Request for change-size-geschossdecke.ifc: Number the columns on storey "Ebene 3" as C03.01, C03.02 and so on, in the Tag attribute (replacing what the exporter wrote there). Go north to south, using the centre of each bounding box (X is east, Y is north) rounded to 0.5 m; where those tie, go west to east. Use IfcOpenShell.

First a look at what the model holds.

```python
import ifcopenshell
import ifcopenshell.util.element
import ifcopenshell.util.placement

model = ifcopenshell.open("change-size-geschossdecke.ifc")
print(model.schema)
storey = next(s for s in model.by_type("IfcBuildingStorey") if s.Name == "Ebene 3")
columns = [e for e in ifcopenshell.util.element.get_decomposition(storey) if e.is_a("IfcColumn")]
for e in sorted(columns, key=lambda e: e.id()):
    origin = ifcopenshell.util.placement.get_local_placement(e.ObjectPlacement)[:3, 3]
    print(e.id(), e.Tag, e.Name, origin.round(2) + 0.0, sep=" | ")
```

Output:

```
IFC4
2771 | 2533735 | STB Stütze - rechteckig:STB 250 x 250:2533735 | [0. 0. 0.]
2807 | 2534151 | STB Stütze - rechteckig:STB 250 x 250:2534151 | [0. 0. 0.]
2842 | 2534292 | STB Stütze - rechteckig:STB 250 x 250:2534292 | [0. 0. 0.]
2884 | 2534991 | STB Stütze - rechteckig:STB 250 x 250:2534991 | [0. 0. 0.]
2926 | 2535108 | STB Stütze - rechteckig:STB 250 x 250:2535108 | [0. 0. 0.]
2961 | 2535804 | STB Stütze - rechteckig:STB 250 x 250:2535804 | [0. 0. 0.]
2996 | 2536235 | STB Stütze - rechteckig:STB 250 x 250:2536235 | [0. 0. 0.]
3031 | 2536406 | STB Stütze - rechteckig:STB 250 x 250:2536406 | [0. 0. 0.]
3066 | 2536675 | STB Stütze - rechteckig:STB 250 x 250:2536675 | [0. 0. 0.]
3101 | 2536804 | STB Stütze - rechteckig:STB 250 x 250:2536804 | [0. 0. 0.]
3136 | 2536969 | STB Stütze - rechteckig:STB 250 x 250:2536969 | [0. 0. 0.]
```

```python
import ifcopenshell
import ifcopenshell.geom
import ifcopenshell.util.element
import ifcopenshell.util.shape

model = ifcopenshell.open("change-size-geschossdecke.ifc")
settings = ifcopenshell.geom.settings()
settings.set("use-world-coords", True)


def centre(element):
    shape = ifcopenshell.geom.create_shape(settings, element)
    return ifcopenshell.util.shape.get_bbox_centroid(shape.geometry)


storey = next(s for s in model.by_type("IfcBuildingStorey") if s.Name == "Ebene 3")
columns = [e for e in ifcopenshell.util.element.get_decomposition(storey) if e.is_a("IfcColumn")]

# Insertion points can sit at a corner or the storey origin, so sort by the geometry (in metres).
centres = {e: centre(e) for e in columns}
columns.sort(key=lambda e: (-round(centres[e][1] / 0.5), centres[e][0]))

for i, e in enumerate(columns, start=1):
    number = f"C03.{i:02d}"
    e.Tag = number
    print(e.id(), number)

model.write("change-size-geschossdecke_edited.ifc")
```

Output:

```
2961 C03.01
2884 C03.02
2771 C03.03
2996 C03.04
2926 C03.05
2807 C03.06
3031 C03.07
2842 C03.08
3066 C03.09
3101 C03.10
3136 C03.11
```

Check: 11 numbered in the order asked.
